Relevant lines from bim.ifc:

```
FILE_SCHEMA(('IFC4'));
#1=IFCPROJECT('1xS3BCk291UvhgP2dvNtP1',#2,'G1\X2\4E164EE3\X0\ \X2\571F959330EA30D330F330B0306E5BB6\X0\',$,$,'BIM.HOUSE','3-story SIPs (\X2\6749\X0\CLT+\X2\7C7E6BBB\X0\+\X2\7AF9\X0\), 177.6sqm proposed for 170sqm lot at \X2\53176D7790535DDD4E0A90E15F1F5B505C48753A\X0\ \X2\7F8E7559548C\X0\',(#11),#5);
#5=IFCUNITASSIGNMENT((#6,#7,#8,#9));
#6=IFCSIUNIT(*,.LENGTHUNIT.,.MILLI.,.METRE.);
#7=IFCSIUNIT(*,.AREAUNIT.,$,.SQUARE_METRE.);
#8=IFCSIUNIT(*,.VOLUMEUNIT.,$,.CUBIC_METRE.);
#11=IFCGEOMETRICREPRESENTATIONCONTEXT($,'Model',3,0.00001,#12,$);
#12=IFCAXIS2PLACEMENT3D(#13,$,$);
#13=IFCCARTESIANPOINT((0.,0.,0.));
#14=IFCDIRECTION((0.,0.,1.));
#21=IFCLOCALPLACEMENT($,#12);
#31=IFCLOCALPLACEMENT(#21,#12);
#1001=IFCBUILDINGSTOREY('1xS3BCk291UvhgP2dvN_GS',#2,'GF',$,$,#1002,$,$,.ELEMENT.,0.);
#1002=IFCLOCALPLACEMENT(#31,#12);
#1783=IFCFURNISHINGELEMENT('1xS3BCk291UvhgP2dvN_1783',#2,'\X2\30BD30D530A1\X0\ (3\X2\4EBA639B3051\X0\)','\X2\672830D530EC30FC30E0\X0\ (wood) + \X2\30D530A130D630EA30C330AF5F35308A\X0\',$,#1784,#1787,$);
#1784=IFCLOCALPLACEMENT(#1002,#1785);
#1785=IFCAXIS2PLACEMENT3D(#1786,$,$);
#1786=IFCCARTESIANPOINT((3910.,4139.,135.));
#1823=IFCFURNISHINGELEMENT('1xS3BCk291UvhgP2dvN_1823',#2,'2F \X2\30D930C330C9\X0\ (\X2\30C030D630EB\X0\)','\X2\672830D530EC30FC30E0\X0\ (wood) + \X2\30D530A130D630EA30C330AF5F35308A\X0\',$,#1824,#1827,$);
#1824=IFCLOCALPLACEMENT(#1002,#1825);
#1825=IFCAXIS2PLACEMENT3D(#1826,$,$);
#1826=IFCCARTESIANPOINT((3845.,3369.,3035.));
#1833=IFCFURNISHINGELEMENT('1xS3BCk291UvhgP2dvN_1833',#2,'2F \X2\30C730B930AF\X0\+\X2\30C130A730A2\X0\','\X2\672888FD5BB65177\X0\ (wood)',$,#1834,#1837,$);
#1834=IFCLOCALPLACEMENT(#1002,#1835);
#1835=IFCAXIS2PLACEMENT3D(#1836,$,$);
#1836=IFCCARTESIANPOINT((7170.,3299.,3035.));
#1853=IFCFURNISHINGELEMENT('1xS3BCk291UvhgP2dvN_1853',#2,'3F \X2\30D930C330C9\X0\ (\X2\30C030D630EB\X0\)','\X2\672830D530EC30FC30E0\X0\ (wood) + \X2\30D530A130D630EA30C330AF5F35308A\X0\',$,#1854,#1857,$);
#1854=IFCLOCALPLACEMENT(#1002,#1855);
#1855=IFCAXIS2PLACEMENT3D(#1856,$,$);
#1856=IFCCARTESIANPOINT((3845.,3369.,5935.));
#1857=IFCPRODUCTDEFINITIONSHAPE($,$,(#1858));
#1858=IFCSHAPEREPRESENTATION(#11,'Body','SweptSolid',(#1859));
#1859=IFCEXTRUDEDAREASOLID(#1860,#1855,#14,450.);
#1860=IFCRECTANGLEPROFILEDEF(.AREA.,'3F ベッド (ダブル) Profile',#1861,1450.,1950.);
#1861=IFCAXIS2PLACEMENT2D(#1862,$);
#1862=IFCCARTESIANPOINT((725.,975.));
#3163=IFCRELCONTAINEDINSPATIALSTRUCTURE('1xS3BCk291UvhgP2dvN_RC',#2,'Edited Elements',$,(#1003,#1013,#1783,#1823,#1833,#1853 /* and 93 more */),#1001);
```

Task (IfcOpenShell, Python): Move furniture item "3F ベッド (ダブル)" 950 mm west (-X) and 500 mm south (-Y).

```python
import ifcopenshell
import ifcopenshell.api.geometry
import ifcopenshell.util.placement
import ifcopenshell.util.unit

model = ifcopenshell.open("bim.ifc")
unit_scale = ifcopenshell.util.unit.calculate_unit_scale(model)

item = model.by_guid("1xS3BCk291UvhgP2dvN_1853")
matrix = ifcopenshell.util.placement.get_local_placement(item.ObjectPlacement)
matrix[0, 3] -= 0.95 / unit_scale
matrix[1, 3] -= 0.5 / unit_scale
ifcopenshell.api.geometry.edit_object_placement(model, product=item, matrix=matrix, is_si=False)

print(ifcopenshell.util.placement.get_local_placement(item.ObjectPlacement).round(3) + 0.0)

model.write("bim_v2.ifc")
```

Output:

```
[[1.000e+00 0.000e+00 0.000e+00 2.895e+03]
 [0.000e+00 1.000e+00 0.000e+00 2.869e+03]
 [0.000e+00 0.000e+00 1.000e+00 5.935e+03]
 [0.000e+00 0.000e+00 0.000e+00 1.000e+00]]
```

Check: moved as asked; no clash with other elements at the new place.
